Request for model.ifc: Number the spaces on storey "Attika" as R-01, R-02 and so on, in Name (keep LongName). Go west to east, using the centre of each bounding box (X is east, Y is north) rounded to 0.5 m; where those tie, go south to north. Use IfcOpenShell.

First a look at what the model holds.

```python
import ifcopenshell
import ifcopenshell.util.element
import ifcopenshell.util.placement

model = ifcopenshell.open("model.ifc")
print(model.schema)
storey = next(s for s in model.by_type("IfcBuildingStorey") if s.Name == "Attika")
spaces = [e for e in ifcopenshell.util.element.get_decomposition(storey) if e.is_a("IfcSpace")]
for e in sorted(spaces, key=lambda e: e.id()):
    origin = ifcopenshell.util.placement.get_local_placement(e.ObjectPlacement)[:3, 3]
    print(e.id(), e.Name, e.LongName, origin.round(2) + 0.0, sep=" | ")
```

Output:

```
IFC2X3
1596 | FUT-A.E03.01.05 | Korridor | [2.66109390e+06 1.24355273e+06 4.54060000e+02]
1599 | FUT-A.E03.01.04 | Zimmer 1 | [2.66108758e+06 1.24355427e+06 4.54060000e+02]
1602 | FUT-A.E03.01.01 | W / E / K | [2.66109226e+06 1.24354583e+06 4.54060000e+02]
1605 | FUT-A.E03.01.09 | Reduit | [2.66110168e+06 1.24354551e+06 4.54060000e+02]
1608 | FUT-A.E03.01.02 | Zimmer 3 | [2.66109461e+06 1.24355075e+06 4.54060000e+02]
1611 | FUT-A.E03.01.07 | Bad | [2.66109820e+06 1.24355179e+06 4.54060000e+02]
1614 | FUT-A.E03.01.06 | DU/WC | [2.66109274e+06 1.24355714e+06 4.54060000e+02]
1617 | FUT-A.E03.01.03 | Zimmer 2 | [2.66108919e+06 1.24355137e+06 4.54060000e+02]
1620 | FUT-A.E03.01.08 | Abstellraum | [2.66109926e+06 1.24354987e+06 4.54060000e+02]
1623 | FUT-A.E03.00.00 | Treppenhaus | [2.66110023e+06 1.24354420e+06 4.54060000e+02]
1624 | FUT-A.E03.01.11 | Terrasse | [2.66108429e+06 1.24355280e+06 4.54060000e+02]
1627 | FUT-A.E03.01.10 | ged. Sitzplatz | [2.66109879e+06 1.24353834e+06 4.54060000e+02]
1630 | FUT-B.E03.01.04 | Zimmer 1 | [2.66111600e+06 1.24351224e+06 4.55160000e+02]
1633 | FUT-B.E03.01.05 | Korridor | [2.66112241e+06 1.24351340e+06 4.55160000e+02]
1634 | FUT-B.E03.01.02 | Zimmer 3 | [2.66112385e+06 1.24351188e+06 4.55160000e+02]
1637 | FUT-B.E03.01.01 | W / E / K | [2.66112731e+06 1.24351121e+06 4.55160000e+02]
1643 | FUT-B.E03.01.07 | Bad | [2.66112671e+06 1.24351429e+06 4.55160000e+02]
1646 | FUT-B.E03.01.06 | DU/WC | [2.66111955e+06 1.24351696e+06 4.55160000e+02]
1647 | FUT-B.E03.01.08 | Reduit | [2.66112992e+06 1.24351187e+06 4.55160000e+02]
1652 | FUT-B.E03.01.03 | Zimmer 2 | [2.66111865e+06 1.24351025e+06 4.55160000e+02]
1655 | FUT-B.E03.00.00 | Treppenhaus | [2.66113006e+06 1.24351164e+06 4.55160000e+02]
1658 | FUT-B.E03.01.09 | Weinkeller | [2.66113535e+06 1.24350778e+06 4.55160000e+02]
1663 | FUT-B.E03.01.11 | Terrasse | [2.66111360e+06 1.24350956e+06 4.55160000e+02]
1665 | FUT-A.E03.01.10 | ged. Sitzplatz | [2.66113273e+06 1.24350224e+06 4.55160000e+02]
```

```python
import ifcopenshell
import ifcopenshell.geom
import ifcopenshell.util.element
import ifcopenshell.util.shape

model = ifcopenshell.open("model.ifc")
settings = ifcopenshell.geom.settings()
settings.set("use-world-coords", True)


def centre(element):
    shape = ifcopenshell.geom.create_shape(settings, element)
    return ifcopenshell.util.shape.get_bbox_centroid(shape.geometry)


storey = next(s for s in model.by_type("IfcBuildingStorey") if s.Name == "Attika")
spaces = [e for e in ifcopenshell.util.element.get_decomposition(storey) if e.is_a("IfcSpace")]

# Insertion points can sit at a corner or the storey origin, so sort by the geometry (in metres).
centres = {e: centre(e) for e in spaces}
spaces.sort(key=lambda e: (round(centres[e][0] / 0.5), centres[e][1]))

for i, e in enumerate(spaces, start=1):
    number = f"R-{i:02d}"
    e.Name = number
    print(e.id(), number)

model.write("model_rev.ifc")
```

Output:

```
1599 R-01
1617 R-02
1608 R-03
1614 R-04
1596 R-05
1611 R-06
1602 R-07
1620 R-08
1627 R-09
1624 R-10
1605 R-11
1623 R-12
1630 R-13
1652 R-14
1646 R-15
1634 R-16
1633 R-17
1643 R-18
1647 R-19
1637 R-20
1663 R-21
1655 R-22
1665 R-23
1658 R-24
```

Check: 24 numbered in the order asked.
